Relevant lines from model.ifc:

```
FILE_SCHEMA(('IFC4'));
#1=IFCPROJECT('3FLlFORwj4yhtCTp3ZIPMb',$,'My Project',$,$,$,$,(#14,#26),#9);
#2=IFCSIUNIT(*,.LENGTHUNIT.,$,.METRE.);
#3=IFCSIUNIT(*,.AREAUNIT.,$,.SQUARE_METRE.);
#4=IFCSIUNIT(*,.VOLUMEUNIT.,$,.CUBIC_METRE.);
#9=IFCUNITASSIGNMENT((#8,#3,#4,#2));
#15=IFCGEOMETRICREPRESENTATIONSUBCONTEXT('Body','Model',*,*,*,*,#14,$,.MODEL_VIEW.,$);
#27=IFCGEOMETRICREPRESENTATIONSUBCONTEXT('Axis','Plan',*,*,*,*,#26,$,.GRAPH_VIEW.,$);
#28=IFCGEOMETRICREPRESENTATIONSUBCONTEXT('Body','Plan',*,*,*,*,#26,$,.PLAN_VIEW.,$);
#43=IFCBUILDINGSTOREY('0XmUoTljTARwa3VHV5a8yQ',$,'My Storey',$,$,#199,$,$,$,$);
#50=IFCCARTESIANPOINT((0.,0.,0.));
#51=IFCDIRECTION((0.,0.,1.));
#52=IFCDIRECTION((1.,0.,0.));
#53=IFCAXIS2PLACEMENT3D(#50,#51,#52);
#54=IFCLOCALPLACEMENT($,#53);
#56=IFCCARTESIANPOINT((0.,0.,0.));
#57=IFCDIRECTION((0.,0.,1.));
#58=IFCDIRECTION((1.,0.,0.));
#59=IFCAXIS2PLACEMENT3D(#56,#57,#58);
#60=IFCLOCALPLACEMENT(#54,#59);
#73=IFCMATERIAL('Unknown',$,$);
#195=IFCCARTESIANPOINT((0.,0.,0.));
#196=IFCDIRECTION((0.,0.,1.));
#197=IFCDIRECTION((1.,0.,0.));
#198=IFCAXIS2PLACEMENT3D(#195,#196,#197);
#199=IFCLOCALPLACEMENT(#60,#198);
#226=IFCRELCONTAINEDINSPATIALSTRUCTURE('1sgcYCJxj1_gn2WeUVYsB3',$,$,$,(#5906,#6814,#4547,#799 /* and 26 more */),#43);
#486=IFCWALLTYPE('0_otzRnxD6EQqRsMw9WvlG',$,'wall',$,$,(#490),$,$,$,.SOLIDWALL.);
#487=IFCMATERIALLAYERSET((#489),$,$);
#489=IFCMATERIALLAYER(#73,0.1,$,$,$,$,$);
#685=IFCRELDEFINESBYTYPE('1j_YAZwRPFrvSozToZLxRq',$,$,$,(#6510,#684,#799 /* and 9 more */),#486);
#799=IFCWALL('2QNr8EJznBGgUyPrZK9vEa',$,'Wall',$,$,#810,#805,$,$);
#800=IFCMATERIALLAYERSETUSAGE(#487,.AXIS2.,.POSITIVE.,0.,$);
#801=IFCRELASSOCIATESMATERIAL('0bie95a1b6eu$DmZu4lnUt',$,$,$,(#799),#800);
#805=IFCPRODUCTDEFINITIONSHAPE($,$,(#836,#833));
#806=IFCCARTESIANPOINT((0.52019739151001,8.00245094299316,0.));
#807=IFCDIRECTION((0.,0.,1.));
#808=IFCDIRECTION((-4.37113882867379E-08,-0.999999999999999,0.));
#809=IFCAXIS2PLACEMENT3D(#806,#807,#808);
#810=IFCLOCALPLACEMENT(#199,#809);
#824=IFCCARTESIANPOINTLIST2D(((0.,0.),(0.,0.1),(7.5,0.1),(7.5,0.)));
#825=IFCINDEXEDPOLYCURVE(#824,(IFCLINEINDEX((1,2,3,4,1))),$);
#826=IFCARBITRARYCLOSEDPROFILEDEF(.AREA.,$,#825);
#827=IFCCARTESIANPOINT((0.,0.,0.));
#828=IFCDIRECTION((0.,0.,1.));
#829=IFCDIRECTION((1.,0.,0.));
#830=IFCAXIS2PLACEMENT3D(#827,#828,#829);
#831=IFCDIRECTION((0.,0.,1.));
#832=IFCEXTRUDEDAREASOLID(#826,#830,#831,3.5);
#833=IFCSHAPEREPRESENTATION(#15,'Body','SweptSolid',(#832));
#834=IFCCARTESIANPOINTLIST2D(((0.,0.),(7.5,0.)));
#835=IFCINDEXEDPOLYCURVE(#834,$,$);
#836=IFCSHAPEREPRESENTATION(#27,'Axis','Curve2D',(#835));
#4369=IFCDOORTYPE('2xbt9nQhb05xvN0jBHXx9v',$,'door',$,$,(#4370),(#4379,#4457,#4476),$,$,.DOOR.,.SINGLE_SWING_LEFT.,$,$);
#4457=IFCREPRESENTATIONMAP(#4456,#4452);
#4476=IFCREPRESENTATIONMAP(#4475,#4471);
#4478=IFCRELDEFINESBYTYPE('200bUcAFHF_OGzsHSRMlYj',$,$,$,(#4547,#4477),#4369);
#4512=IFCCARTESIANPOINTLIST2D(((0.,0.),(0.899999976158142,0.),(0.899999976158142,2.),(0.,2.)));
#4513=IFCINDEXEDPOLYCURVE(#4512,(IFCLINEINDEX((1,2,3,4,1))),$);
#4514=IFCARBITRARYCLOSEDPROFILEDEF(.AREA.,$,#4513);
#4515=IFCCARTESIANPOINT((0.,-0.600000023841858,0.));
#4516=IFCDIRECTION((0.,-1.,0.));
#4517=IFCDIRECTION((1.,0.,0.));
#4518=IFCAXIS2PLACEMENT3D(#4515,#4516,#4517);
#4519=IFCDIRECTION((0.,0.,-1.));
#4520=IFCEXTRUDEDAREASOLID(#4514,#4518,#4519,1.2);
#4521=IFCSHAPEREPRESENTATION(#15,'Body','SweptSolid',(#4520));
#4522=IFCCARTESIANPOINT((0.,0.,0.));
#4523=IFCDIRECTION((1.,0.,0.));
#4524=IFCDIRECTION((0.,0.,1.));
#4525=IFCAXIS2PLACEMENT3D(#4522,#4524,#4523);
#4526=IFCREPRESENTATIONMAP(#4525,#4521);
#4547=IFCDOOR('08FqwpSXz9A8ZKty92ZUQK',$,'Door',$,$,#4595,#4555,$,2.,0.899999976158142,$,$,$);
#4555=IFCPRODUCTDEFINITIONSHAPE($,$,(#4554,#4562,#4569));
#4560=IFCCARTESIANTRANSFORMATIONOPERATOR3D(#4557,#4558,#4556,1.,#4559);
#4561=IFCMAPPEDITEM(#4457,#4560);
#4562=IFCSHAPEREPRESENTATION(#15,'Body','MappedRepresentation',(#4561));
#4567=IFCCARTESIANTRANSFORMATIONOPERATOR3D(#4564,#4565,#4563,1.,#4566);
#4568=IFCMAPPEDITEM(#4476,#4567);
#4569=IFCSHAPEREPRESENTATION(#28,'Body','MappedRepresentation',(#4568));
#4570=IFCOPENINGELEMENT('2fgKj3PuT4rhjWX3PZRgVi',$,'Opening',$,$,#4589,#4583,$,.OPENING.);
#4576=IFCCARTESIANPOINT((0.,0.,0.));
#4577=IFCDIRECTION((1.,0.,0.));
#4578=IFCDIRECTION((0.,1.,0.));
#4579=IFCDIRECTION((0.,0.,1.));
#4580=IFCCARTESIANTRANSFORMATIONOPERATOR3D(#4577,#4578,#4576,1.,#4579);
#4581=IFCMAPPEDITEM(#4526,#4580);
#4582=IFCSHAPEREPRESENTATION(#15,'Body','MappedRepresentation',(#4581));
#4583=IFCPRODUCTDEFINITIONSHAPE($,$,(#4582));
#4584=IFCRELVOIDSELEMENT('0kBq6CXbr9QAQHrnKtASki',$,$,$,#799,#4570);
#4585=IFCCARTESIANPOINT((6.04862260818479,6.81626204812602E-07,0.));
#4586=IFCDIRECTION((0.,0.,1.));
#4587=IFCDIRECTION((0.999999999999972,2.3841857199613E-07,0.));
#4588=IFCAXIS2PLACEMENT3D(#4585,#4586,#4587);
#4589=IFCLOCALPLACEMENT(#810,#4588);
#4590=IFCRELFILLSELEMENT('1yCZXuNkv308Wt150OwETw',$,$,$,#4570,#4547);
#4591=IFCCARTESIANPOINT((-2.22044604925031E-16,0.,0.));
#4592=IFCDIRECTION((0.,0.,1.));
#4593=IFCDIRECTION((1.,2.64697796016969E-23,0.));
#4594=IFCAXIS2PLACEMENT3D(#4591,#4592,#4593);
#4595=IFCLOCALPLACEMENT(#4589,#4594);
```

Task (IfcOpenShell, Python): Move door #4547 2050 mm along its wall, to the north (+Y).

```python
import ifcopenshell
import ifcopenshell.api.geometry
import ifcopenshell.util.placement
import ifcopenshell.util.unit

model = ifcopenshell.open("model.ifc")
unit_scale = ifcopenshell.util.unit.calculate_unit_scale(model)

door = model.by_guid("08FqwpSXz9A8ZKty92ZUQK")
opening = door.FillsVoids[0].RelatingOpeningElement
wall = opening.VoidsElements[0].RelatingBuildingElement

wall_matrix = ifcopenshell.util.placement.get_local_placement(wall.ObjectPlacement)
shift = wall_matrix[:3, 0] * -2.05 / unit_scale
before = ifcopenshell.util.placement.get_local_placement(door.ObjectPlacement)[:3, 3].copy()

# The door is placed relative to its opening, so it follows when the opening moves.
matrix = ifcopenshell.util.placement.get_local_placement(opening.ObjectPlacement)
matrix[:3, 3] += shift
ifcopenshell.api.geometry.edit_object_placement(
    model, product=opening, matrix=matrix, is_si=False, should_transform_children=True
)

after = ifcopenshell.util.placement.get_local_placement(door.ObjectPlacement)[:3, 3]
print("door moved by", (after - before).round(3) + 0.0)

model.write("model-out.ifc")
```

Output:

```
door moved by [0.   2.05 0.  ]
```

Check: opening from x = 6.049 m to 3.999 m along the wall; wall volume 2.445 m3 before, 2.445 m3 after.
